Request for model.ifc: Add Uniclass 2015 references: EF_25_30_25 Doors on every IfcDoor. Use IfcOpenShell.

First a look at what the model holds.

```python
import ifcopenshell

model = ifcopenshell.open("model.ifc")
print(model.schema)
print("classifications:", [c.Name for c in model.by_type("IfcClassification")])
for ifc_class in ("IfcDoor", "IfcRoof", "IfcStair", "IfcWall", "IfcWindow"):
    print(ifc_class, len(model.by_type(ifc_class)))
```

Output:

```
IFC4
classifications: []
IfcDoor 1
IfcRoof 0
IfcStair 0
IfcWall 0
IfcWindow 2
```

```python
import ifcopenshell
import ifcopenshell.api.classification

model = ifcopenshell.open("model.ifc")

system = ifcopenshell.api.classification.add_classification(model, classification="Uniclass 2015")

codes = {
    "IfcDoor": ("EF_25_30_25", "Doors"),
}
for ifc_class, (code, name) in codes.items():
    products = model.by_type(ifc_class)
    ifcopenshell.api.classification.add_reference(
        model, products=products, classification=system, identification=code, name=name
    )
    print(code, len(products))

model.write("model-out.ifc")
```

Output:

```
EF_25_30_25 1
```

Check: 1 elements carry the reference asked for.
